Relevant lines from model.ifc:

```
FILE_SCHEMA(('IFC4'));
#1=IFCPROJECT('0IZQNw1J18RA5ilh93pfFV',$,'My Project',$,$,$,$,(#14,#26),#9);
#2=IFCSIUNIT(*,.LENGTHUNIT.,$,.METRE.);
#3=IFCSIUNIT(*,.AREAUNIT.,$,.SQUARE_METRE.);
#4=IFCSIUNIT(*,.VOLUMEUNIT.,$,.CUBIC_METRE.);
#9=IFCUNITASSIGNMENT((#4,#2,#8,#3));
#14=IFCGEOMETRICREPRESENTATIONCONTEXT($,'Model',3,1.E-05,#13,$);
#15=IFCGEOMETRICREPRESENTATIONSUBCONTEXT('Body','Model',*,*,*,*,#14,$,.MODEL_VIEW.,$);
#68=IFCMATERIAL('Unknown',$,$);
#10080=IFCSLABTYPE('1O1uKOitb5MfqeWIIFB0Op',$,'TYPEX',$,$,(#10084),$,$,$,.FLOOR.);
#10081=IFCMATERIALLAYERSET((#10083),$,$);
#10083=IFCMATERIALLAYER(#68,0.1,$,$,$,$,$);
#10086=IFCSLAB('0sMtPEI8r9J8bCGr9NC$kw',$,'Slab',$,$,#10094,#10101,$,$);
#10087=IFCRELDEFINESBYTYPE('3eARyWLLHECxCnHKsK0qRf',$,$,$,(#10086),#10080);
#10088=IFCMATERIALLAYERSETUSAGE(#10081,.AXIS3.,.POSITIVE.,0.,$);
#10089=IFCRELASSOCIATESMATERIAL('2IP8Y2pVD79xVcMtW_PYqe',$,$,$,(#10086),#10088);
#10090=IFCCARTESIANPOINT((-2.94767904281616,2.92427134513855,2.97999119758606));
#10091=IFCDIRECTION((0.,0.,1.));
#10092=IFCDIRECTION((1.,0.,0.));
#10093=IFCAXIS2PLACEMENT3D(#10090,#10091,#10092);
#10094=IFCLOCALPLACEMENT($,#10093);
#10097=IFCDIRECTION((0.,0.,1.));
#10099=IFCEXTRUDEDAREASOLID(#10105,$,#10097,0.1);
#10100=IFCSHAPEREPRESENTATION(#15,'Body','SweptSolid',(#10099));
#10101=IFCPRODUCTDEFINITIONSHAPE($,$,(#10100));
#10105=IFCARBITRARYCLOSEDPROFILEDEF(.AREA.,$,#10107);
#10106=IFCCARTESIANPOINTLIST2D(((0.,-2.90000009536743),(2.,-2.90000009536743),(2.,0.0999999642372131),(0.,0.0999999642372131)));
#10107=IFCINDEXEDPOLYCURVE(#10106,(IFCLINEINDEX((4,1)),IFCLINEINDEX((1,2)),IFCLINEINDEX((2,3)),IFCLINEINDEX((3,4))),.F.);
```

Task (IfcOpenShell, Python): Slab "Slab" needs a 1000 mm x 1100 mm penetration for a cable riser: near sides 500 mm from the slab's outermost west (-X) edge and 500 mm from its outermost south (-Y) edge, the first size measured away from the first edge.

```python
import numpy as np
import ifcopenshell
import ifcopenshell.api.feature
import ifcopenshell.api.geometry
import ifcopenshell.api.root
import ifcopenshell.geom
import ifcopenshell.util.placement
import ifcopenshell.util.representation
import ifcopenshell.util.shape
import ifcopenshell.util.unit

model = ifcopenshell.open("model.ifc")
unit_scale = ifcopenshell.util.unit.calculate_unit_scale(model)
settings = ifcopenshell.geom.settings()


def volume(element):
    """Net volume in cubic metres, openings subtracted."""
    shape = ifcopenshell.geom.create_shape(settings, element)
    return ifcopenshell.util.shape.get_volume(shape.geometry)


slab = model.by_guid("0sMtPEI8r9J8bCGr9NC$kw")
before = volume(slab)

# Extent in the slab's own axes, in metres. The edges named are its -X and -Y sides.
slab_shape = ifcopenshell.geom.create_shape(settings, slab)
vertices = ifcopenshell.util.shape.get_vertices(slab_shape.geometry)
x_min, y_min, bottom = vertices.min(axis=0)
top = vertices[:, 2].max()

opening = ifcopenshell.api.root.create_entity(model, ifc_class="IfcOpeningElement", name="Cable riser opening", predefined_type="OPENING")
context = ifcopenshell.util.representation.get_context(model, "Model", "Body", "MODEL_VIEW")
width, depth = 1, 1.1
outline = [(0.0, 0.0), (width, 0.0), (width, depth), (0.0, depth), (0.0, 0.0)]
# Overshoot both faces by 50 mm so the cut is clean.
shape = ifcopenshell.api.geometry.add_slab_representation(
    model, context=context, depth=top - bottom + 0.1, polyline=outline
)
ifcopenshell.api.geometry.assign_representation(model, product=opening, representation=shape)

matrix = ifcopenshell.util.placement.get_local_placement(slab.ObjectPlacement)
matrix[:, 3] = matrix @ np.append(np.array([x_min + 0.5, y_min + 0.5, bottom - 0.05]) / unit_scale, 1.0)
ifcopenshell.api.geometry.edit_object_placement(model, product=opening, matrix=matrix, is_si=False)
ifcopenshell.api.feature.add_feature(model, feature=opening, element=slab)

after = volume(slab)

print(f"slab volume {before:.3f} -> {after:.3f} m3")

model.write("model_rev.ifc")
```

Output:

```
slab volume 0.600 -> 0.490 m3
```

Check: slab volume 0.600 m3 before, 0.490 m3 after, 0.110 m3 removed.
